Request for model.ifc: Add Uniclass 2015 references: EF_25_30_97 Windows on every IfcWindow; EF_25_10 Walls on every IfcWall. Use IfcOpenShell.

First a look at what the model holds.

```python
import ifcopenshell

model = ifcopenshell.open("model.ifc")
print(model.schema)
print("classifications:", [c.Name for c in model.by_type("IfcClassification")])
for ifc_class in ("IfcDoor", "IfcRoof", "IfcStair", "IfcWall", "IfcWindow"):
    print(ifc_class, len(model.by_type(ifc_class)))
```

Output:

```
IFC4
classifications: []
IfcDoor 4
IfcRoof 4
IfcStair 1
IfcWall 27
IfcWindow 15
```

```python
import ifcopenshell
import ifcopenshell.api.classification

model = ifcopenshell.open("model.ifc")

system = ifcopenshell.api.classification.add_classification(model, classification="Uniclass 2015")

codes = {
    "IfcWindow": ("EF_25_30_97", "Windows"),
    "IfcWall": ("EF_25_10", "Walls"),
}
for ifc_class, (code, name) in codes.items():
    products = model.by_type(ifc_class)
    ifcopenshell.api.classification.add_reference(
        model, products=products, classification=system, identification=code, name=name
    )
    print(code, len(products))

model.write("model_edited.ifc")
```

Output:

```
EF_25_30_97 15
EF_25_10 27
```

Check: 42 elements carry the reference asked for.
